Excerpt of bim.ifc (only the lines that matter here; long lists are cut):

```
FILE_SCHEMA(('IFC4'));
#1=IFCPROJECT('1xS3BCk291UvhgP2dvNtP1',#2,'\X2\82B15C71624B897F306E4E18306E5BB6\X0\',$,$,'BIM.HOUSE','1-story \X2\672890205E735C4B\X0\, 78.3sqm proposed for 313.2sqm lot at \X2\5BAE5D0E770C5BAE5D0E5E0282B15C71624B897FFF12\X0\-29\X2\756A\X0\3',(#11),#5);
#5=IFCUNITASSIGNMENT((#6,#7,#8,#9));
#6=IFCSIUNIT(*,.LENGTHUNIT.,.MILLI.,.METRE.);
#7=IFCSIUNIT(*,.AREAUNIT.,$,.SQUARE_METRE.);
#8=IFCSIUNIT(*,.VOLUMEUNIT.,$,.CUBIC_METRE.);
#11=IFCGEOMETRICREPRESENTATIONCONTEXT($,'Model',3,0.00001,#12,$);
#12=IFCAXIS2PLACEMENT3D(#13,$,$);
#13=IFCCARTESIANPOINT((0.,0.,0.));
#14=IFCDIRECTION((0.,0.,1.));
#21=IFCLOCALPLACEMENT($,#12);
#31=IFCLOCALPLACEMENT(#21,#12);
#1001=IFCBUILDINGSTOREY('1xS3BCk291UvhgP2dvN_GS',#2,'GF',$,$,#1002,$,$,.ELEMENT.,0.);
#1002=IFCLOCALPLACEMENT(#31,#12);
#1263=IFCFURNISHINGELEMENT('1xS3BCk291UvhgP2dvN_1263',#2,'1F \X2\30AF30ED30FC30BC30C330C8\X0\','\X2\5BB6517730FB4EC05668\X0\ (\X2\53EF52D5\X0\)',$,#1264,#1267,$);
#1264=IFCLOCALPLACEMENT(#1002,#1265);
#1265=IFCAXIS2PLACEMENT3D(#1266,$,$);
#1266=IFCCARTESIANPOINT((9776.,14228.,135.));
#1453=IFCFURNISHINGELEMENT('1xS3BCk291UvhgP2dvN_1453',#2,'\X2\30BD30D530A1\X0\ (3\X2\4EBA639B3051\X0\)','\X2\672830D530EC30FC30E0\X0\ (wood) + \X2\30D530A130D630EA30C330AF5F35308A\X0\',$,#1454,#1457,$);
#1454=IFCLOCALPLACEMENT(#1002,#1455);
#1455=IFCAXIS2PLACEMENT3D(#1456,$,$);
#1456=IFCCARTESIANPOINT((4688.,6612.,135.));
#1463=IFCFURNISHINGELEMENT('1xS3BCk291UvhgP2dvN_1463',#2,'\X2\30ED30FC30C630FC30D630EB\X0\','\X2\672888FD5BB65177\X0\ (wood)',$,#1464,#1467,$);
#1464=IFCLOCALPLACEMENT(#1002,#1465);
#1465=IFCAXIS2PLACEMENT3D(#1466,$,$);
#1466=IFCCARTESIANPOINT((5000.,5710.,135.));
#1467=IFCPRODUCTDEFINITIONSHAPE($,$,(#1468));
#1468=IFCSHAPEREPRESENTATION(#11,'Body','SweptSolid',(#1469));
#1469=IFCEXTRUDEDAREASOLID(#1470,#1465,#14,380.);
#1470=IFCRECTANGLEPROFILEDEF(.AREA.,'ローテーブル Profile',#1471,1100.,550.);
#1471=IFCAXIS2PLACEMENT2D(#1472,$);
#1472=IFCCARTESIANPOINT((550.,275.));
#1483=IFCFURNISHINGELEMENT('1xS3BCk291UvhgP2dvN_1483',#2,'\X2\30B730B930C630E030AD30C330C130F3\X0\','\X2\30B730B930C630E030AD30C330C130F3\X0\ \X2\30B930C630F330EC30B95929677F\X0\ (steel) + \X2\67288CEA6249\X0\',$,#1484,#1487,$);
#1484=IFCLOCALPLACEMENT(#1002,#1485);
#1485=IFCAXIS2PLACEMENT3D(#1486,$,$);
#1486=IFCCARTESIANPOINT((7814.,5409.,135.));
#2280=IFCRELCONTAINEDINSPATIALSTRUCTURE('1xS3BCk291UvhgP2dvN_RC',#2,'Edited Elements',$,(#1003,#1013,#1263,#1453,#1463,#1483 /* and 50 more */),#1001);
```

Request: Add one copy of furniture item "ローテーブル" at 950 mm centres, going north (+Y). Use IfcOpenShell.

```python
import numpy as np
import ifcopenshell
import ifcopenshell.api.geometry
import ifcopenshell.api.root
import ifcopenshell.util.element
import ifcopenshell.util.placement

model = ifcopenshell.open("bim.ifc")


def reuse_history(source, copy):
    """copy_class also copies each property set's owner history, people and application; keep the originals."""
    for rel in copy.IsDefinedBy:
        if rel.is_a("IfcRelDefinesByProperties") and (history := rel.RelatingPropertyDefinition.OwnerHistory):
            rel.RelatingPropertyDefinition.OwnerHistory = source.OwnerHistory
            ifcopenshell.util.element.remove_deep2(model, history)


source = model.by_id(1463)
base = ifcopenshell.util.placement.get_local_placement(source.ObjectPlacement)
step = np.array([0.0, 1.0, 0.0]) * 950.0

for i in range(1, 2):
    copy = ifcopenshell.api.root.copy_class(model, product=source)
    copy.Representation = ifcopenshell.util.element.copy_deep(
        model, source.Representation, exclude=["IfcGeometricRepresentationContext", "IfcRepresentationMap"]
    )
    reuse_history(source, copy)
    matrix = base.copy()
    matrix[:3, 3] += i * step
    print("added at", matrix[:3, 3].round(3) + 0.0)
    ifcopenshell.api.geometry.edit_object_placement(model, product=copy, matrix=matrix, is_si=False)

model.write("bim_edited.ifc")
```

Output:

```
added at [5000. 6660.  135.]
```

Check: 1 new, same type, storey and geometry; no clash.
